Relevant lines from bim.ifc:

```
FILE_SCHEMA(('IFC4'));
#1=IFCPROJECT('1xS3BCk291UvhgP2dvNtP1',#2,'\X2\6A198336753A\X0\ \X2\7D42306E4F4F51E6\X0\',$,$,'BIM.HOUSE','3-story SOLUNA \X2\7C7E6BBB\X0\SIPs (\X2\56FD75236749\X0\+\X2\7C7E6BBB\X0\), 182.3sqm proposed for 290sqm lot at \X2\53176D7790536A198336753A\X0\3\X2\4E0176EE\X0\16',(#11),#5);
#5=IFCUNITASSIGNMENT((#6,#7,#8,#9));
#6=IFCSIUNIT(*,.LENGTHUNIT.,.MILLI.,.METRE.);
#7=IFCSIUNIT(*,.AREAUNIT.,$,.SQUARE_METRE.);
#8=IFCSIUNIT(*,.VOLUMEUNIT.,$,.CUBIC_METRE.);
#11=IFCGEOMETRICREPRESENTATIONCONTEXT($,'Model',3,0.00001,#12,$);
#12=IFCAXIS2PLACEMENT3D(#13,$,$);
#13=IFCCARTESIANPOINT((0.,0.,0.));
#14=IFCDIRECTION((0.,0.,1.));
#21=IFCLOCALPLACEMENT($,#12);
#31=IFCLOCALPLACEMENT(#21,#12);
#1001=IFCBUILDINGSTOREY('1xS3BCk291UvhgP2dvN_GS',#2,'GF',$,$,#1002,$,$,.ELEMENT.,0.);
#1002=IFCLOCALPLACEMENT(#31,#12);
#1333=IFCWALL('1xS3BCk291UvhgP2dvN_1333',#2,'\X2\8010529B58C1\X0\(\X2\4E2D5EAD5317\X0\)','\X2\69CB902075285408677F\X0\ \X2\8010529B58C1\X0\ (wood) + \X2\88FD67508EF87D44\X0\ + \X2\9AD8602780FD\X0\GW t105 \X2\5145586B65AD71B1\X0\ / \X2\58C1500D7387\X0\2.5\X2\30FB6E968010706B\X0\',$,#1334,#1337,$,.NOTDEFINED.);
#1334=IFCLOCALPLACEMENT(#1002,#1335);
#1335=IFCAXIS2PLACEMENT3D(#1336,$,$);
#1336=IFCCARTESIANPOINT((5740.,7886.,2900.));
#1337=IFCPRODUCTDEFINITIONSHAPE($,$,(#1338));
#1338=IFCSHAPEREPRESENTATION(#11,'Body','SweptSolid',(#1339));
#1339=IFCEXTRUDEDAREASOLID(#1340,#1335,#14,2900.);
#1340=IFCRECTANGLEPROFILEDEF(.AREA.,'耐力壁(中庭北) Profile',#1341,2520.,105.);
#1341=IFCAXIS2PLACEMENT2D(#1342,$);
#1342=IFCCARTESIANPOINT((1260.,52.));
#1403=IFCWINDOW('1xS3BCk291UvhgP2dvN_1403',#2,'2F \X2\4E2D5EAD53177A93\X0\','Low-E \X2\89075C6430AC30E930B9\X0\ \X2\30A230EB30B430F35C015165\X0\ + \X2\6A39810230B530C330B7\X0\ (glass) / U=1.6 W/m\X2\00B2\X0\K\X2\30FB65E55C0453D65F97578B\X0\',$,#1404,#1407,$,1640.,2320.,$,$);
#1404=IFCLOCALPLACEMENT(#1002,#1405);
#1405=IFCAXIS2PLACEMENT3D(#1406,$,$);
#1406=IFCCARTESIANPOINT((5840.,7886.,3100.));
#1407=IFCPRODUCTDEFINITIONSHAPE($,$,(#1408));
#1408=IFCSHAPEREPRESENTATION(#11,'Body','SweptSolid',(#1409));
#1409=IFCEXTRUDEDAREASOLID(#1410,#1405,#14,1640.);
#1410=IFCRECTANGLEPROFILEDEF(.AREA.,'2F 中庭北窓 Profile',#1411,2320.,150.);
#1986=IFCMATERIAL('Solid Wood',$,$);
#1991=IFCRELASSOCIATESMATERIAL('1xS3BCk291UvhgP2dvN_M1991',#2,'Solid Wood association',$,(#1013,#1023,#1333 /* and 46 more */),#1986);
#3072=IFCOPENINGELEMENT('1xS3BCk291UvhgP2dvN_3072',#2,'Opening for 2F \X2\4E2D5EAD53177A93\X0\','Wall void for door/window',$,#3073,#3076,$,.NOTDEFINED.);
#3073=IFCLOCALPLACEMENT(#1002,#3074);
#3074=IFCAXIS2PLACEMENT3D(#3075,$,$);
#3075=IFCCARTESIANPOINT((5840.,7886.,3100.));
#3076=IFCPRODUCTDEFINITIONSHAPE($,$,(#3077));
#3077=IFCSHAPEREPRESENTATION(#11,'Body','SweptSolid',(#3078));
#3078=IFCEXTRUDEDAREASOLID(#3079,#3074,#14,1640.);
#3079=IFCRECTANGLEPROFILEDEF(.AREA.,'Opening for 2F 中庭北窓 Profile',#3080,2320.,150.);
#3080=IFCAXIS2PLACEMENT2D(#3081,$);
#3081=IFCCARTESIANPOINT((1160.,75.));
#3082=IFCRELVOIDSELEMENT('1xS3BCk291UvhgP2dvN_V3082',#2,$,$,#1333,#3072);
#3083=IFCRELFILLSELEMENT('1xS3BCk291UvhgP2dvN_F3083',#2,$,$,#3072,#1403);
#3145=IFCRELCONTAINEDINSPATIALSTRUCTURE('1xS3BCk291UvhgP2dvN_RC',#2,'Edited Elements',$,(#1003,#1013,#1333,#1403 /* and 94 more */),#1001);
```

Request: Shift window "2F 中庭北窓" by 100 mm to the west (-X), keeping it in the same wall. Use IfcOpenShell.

```python
import ifcopenshell
import ifcopenshell.api.geometry
import ifcopenshell.util.placement
import ifcopenshell.util.unit

model = ifcopenshell.open("bim.ifc")
unit_scale = ifcopenshell.util.unit.calculate_unit_scale(model)

window = model.by_guid("1xS3BCk291UvhgP2dvN_1403")
opening = window.FillsVoids[0].RelatingOpeningElement
wall = opening.VoidsElements[0].RelatingBuildingElement

wall_matrix = ifcopenshell.util.placement.get_local_placement(wall.ObjectPlacement)
shift = wall_matrix[:3, 0] * -0.1 / unit_scale
before = ifcopenshell.util.placement.get_local_placement(window.ObjectPlacement)[:3, 3].copy()

# The window is not placed relative to its opening, so move both.
for product in (opening, window):
    matrix = ifcopenshell.util.placement.get_local_placement(product.ObjectPlacement)
    matrix[:3, 3] += shift
    ifcopenshell.api.geometry.edit_object_placement(model, product=product, matrix=matrix, is_si=False)

after = ifcopenshell.util.placement.get_local_placement(window.ObjectPlacement)[:3, 3]
print("window moved by", (after - before).round(3) + 0.0)

model.write("bim_edited.ifc")
```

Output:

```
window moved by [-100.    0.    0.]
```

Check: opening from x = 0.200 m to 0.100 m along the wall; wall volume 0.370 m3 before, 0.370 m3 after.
